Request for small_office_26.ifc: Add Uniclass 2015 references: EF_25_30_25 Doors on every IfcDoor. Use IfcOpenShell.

First a look at what the model holds.

```python
import ifcopenshell

model = ifcopenshell.open("small_office_26.ifc")
print(model.schema)
print("classifications:", [c.Name for c in model.by_type("IfcClassification")])
for ifc_class in ("IfcDoor", "IfcRoof", "IfcStair", "IfcWall", "IfcWindow"):
    print(ifc_class, len(model.by_type(ifc_class)))
```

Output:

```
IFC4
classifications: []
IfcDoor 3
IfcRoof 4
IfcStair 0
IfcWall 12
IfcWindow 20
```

```python
import ifcopenshell
import ifcopenshell.api.classification

model = ifcopenshell.open("small_office_26.ifc")

system = ifcopenshell.api.classification.add_classification(model, classification="Uniclass 2015")

codes = {
    "IfcDoor": ("EF_25_30_25", "Doors"),
}
for ifc_class, (code, name) in codes.items():
    products = model.by_type(ifc_class)
    ifcopenshell.api.classification.add_reference(
        model, products=products, classification=system, identification=code, name=name
    )
    print(code, len(products))

model.write("small_office_26_rev.ifc")
```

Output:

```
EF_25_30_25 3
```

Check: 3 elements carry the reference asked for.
